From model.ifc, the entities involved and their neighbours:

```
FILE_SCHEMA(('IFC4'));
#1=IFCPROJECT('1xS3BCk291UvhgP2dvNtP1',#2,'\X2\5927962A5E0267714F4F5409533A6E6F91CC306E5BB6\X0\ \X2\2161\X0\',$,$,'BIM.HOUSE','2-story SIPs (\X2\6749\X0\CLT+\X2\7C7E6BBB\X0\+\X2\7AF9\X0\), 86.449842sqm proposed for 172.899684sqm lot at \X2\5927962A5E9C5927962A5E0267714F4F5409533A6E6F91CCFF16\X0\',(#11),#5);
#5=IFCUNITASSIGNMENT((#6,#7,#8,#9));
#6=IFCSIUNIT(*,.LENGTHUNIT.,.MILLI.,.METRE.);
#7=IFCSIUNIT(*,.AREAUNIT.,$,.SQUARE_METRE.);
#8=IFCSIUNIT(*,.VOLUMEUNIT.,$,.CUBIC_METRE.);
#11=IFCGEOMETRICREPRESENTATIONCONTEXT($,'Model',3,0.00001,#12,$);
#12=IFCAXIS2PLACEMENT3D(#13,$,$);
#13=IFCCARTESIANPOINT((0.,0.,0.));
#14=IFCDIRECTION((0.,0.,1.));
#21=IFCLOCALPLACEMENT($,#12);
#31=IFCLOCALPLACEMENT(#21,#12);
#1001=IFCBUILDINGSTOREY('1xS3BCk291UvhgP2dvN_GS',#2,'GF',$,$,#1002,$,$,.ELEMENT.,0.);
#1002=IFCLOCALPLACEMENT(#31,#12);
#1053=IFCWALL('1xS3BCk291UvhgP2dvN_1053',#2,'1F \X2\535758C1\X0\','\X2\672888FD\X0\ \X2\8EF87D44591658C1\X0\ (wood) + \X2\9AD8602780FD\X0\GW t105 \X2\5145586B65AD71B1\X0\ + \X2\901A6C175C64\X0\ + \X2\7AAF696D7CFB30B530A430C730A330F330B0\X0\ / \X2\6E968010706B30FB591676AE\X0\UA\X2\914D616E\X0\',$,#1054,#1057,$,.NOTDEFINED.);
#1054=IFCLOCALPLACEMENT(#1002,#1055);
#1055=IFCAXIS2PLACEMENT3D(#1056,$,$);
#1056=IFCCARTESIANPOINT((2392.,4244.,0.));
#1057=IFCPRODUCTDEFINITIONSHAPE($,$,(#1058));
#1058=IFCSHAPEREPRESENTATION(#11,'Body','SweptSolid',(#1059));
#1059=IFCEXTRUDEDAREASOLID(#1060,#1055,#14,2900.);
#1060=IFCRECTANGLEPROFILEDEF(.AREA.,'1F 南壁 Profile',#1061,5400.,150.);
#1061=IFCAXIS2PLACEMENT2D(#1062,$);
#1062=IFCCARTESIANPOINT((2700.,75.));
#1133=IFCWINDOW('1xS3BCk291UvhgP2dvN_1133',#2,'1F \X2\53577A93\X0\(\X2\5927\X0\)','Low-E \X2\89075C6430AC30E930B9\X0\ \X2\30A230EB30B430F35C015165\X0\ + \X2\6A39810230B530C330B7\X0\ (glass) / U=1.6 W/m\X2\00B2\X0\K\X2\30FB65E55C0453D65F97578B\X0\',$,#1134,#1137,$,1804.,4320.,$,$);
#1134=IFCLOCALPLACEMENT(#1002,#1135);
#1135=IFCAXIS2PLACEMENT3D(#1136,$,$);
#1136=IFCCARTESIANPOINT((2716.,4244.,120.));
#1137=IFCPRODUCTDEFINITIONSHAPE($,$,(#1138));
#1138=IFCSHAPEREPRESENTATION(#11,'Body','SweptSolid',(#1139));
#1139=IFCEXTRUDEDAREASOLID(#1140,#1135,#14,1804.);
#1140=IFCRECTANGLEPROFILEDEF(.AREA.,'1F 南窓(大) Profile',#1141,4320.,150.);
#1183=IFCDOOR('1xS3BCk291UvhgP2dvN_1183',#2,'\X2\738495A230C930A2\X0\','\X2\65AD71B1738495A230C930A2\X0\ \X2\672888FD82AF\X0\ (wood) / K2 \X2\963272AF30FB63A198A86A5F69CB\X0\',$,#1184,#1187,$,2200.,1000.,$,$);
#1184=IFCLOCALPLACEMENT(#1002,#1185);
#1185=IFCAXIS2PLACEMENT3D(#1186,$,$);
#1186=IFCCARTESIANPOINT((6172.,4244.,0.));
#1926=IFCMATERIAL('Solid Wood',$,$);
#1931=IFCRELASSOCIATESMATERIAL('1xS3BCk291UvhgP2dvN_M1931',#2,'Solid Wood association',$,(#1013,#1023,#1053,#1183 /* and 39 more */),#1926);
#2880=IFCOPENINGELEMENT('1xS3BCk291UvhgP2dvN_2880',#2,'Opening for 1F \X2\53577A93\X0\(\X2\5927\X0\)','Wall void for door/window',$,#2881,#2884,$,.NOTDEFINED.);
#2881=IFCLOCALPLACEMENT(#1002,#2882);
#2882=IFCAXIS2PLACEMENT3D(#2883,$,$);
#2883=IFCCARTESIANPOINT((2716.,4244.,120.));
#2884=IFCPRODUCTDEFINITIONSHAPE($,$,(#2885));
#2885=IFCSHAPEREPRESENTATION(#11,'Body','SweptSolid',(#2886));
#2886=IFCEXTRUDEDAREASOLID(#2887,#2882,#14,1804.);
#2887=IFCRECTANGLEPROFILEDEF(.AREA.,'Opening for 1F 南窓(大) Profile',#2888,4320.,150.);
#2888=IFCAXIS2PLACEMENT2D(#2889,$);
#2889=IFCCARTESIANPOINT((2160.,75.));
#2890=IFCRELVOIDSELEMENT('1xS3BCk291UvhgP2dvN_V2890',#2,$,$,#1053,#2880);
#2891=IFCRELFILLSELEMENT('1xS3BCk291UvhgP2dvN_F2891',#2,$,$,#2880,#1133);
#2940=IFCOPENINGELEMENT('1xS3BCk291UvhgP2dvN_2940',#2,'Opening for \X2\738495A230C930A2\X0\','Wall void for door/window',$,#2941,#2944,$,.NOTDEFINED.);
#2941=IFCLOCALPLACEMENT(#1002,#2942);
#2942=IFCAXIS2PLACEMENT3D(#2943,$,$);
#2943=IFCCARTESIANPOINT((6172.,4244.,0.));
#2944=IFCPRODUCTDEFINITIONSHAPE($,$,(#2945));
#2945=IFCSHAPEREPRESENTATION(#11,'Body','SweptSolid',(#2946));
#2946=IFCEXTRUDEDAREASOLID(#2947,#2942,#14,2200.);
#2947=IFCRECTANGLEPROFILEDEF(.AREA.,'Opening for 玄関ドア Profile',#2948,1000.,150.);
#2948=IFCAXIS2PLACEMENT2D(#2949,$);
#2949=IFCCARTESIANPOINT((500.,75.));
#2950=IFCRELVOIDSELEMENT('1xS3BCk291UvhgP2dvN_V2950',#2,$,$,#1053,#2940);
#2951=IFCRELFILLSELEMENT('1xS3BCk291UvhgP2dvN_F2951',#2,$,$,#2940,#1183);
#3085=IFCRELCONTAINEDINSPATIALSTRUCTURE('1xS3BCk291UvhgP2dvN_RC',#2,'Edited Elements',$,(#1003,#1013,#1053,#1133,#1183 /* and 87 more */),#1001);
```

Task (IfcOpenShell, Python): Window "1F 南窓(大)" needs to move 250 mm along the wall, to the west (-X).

```python
import ifcopenshell
import ifcopenshell.api.geometry
import ifcopenshell.util.placement

model = ifcopenshell.open("model.ifc")

window = model.by_guid("1xS3BCk291UvhgP2dvN_1133")
opening = window.FillsVoids[0].RelatingOpeningElement
wall = opening.VoidsElements[0].RelatingBuildingElement

wall_matrix = ifcopenshell.util.placement.get_local_placement(wall.ObjectPlacement)
shift = wall_matrix[:3, 0] * -250.0
before = ifcopenshell.util.placement.get_local_placement(window.ObjectPlacement)[:3, 3].copy()

# The window is not placed relative to its opening, so move both.
for product in (opening, window):
    matrix = ifcopenshell.util.placement.get_local_placement(product.ObjectPlacement)
    matrix[:3, 3] += shift
    ifcopenshell.api.geometry.edit_object_placement(model, product=product, matrix=matrix, is_si=False)

after = ifcopenshell.util.placement.get_local_placement(window.ObjectPlacement)[:3, 3]
print("window moved by", (after - before).round(3) + 0.0)

model.write("model_v2.ifc")
```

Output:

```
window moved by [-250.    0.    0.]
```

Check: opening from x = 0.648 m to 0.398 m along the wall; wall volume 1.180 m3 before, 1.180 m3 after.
